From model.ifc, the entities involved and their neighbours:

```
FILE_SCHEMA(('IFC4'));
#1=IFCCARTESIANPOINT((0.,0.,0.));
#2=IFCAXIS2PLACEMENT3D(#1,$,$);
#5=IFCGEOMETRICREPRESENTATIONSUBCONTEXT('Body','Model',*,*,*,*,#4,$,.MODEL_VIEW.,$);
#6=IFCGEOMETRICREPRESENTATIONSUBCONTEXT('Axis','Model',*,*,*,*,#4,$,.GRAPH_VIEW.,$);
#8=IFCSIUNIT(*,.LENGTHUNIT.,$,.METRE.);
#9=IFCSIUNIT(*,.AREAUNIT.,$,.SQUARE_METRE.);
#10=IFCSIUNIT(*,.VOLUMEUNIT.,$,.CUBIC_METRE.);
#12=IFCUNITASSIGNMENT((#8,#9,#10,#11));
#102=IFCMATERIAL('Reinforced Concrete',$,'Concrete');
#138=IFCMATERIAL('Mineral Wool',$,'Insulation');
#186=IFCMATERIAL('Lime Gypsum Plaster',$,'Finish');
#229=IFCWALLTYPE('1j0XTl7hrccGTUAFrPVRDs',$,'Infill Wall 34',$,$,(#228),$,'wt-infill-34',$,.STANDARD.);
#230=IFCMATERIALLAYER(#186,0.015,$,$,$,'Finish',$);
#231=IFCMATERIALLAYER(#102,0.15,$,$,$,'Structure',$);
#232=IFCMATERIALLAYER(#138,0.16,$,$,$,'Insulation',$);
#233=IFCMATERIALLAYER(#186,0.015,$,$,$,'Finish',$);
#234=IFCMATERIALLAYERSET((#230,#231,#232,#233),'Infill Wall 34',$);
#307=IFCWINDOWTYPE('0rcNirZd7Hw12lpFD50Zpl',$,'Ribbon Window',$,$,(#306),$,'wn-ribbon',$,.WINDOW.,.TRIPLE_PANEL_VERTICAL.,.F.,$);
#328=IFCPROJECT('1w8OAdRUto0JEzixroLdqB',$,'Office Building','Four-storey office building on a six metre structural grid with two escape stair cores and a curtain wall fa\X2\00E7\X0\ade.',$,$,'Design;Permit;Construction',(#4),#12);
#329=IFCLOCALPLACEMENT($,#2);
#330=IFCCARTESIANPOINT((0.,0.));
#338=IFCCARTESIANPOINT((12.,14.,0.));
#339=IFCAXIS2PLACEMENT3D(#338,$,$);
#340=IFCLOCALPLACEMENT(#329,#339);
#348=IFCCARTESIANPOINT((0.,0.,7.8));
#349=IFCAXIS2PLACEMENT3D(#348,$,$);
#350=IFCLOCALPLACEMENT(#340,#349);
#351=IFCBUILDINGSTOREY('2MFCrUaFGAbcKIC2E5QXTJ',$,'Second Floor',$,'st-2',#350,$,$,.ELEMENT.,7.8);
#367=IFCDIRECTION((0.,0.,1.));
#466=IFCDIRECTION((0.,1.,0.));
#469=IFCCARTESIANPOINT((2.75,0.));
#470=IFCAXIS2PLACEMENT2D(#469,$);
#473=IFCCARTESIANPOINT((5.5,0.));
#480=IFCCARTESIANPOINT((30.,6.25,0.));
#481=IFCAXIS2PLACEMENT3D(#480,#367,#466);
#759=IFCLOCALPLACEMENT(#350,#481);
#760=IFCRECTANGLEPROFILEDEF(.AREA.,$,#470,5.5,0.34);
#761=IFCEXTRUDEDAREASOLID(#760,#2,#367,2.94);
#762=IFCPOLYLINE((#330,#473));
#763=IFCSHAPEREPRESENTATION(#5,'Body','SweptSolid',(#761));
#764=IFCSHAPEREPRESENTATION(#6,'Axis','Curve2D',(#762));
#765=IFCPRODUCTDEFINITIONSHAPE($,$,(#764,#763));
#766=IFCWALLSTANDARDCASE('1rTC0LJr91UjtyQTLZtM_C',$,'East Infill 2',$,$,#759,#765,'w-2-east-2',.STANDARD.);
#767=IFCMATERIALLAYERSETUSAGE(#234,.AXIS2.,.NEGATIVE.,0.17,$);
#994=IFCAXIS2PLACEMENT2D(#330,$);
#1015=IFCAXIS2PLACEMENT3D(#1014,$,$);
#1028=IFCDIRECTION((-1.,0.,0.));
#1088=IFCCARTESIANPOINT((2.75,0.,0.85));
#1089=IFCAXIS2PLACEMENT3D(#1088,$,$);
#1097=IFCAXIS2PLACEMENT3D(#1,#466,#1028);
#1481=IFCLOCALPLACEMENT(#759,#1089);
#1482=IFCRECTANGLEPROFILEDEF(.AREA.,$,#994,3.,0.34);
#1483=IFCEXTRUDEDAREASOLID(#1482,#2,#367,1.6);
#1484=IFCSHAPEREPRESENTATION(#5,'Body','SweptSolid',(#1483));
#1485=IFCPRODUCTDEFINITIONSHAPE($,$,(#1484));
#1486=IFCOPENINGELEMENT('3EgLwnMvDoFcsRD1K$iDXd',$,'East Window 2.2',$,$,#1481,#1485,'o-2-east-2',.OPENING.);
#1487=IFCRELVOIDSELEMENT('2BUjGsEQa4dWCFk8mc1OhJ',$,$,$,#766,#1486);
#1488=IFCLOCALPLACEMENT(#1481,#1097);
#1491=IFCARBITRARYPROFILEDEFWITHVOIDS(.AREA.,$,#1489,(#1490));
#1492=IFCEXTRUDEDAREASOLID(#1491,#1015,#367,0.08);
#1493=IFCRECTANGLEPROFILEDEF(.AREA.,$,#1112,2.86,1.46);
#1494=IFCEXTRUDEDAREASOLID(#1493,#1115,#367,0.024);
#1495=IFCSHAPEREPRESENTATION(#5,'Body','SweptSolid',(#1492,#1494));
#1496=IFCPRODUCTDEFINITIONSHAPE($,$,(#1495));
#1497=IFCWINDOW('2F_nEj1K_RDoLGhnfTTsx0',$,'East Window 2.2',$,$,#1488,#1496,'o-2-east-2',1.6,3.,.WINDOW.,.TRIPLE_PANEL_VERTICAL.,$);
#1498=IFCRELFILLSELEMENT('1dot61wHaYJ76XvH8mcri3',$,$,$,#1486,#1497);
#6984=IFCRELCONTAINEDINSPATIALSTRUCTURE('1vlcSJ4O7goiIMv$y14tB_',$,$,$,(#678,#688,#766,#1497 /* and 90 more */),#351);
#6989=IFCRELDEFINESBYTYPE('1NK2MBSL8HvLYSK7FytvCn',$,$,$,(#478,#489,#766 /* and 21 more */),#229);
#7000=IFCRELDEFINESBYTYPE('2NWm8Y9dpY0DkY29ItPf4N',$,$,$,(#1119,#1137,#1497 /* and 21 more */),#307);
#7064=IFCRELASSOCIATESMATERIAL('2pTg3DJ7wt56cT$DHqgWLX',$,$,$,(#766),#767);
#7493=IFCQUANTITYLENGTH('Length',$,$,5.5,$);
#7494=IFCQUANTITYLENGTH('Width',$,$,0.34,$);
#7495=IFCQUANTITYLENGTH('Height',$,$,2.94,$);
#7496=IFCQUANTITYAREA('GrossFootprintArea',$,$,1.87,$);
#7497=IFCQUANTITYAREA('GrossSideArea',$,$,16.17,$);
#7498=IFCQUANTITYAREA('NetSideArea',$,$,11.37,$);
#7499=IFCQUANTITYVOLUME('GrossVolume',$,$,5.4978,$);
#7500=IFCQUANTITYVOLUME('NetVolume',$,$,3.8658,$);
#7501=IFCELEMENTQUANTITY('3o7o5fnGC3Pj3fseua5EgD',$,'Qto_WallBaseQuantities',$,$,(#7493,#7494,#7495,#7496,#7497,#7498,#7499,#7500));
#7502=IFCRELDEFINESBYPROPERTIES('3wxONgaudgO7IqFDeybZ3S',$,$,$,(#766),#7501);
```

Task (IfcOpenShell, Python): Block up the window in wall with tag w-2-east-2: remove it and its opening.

```python
import ifcopenshell
import ifcopenshell.api.feature
import ifcopenshell.api.pset
import ifcopenshell.api.root
import ifcopenshell.geom
import ifcopenshell.util.element
import ifcopenshell.util.shape
import ifcopenshell.util.unit

model = ifcopenshell.open("model.ifc")
area_scale = ifcopenshell.util.unit.calculate_unit_scale(model, "AREAUNIT")
volume_scale = ifcopenshell.util.unit.calculate_unit_scale(model, "VOLUMEUNIT")
settings = ifcopenshell.geom.settings()


def volume(element):
    """Net volume in cubic metres, openings subtracted."""
    shape = ifcopenshell.geom.create_shape(settings, element)
    return ifcopenshell.util.shape.get_volume(shape.geometry)


window = model.by_guid("2F_nEj1K_RDoLGhnfTTsx0")
opening = window.FillsVoids[0].RelatingOpeningElement
wall = opening.VoidsElements[0].RelatingBuildingElement
before = volume(wall)

ifcopenshell.api.root.remove_product(model, product=window)
ifcopenshell.api.feature.remove_feature(model, feature=opening)

after = volume(wall)
thickness = 0.34  # wall thickness in metres

# Update the wall's stored quantities.
qto = model.by_id(ifcopenshell.util.element.get_pset(wall, "Qto_WallBaseQuantities", should_inherit=False)["id"])
ifcopenshell.api.pset.edit_qto(model, qto=qto, properties={
    "NetSideArea": after / thickness / area_scale,
    "NetVolume": after / volume_scale,
})

print(f"wall volume {before:.3f} -> {after:.3f} m3")

model.write("model_v2.ifc")
```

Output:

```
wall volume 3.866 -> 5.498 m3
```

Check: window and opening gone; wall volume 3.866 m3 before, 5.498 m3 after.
